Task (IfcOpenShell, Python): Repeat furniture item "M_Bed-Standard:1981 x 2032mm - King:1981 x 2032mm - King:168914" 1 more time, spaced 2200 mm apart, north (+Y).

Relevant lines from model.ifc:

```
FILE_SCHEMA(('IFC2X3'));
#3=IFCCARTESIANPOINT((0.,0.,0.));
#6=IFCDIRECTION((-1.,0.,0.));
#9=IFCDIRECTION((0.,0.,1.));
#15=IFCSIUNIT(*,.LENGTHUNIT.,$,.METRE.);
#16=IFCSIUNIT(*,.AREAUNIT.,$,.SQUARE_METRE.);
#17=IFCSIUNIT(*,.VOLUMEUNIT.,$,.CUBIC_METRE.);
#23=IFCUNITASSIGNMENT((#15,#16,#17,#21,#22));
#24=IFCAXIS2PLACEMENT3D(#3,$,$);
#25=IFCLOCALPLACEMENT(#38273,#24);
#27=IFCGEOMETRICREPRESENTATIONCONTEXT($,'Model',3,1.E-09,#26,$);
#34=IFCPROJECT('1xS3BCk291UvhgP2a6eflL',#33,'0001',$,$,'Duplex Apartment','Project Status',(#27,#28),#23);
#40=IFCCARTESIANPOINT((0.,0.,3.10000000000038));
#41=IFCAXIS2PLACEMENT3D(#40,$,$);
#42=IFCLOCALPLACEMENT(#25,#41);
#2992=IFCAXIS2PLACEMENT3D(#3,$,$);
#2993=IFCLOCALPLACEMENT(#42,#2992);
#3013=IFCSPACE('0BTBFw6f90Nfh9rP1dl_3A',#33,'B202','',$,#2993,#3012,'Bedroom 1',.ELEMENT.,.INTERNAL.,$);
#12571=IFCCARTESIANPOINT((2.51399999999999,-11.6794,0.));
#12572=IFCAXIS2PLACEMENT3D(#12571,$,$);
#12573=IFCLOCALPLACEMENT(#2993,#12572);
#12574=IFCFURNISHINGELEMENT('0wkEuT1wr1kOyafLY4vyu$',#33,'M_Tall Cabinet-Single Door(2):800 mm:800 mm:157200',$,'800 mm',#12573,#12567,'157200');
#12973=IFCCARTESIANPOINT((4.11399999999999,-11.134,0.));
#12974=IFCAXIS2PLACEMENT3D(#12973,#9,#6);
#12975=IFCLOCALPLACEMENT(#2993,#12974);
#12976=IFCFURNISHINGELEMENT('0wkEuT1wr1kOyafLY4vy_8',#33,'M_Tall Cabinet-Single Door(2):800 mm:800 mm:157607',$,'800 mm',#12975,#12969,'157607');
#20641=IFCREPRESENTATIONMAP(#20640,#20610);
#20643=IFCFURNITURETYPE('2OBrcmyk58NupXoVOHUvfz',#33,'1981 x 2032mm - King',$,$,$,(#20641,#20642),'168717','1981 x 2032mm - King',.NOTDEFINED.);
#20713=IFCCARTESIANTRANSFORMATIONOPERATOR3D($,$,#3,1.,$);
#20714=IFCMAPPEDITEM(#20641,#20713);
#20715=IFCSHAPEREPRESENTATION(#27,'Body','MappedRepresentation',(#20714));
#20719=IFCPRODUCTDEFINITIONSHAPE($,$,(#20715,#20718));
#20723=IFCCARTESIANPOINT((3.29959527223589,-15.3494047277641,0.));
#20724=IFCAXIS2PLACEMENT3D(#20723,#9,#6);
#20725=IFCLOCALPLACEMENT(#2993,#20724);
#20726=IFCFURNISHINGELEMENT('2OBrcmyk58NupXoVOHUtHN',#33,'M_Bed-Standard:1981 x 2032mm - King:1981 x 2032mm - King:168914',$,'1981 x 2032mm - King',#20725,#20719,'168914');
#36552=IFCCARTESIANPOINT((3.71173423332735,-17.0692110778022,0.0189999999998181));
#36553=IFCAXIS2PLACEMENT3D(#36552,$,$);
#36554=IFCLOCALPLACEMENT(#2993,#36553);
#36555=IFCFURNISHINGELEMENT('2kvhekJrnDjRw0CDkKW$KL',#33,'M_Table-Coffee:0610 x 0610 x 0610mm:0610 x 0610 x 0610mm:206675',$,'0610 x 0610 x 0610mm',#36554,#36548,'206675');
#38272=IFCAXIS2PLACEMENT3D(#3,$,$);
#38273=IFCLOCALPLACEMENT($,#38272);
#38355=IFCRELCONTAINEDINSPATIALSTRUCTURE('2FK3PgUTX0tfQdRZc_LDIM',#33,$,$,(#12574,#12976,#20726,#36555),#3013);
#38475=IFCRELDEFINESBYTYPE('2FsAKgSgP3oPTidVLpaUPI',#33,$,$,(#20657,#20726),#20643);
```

```python
import numpy as np
import ifcopenshell
import ifcopenshell.api.geometry
import ifcopenshell.api.root
import ifcopenshell.util.element
import ifcopenshell.util.placement

model = ifcopenshell.open("model.ifc")


def reuse_history(source, copy):
    """copy_class also copies each property set's owner history, people and application; keep the originals."""
    for rel in copy.IsDefinedBy:
        if rel.is_a("IfcRelDefinesByProperties") and (history := rel.RelatingPropertyDefinition.OwnerHistory):
            rel.RelatingPropertyDefinition.OwnerHistory = source.OwnerHistory
            ifcopenshell.util.element.remove_deep2(model, history)


source = model.by_guid("2OBrcmyk58NupXoVOHUtHN")
base = ifcopenshell.util.placement.get_local_placement(source.ObjectPlacement)
step = np.array([0.0, 1.0, 0.0]) * 2.2

for i in range(1, 2):
    copy = ifcopenshell.api.root.copy_class(model, product=source)
    copy.Representation = ifcopenshell.util.element.copy_deep(
        model, source.Representation, exclude=["IfcGeometricRepresentationContext", "IfcRepresentationMap"]
    )
    copy.Name = "M_Bed-Standard:1981 x 2032mm - King:1981 x 2032mm - King"
    copy.Tag = None
    reuse_history(source, copy)
    matrix = base.copy()
    matrix[:3, 3] += i * step
    print("added at", matrix[:3, 3].round(3) + 0.0)
    ifcopenshell.api.geometry.edit_object_placement(model, product=copy, matrix=matrix, is_si=False)

model.write("model_rev.ifc")
```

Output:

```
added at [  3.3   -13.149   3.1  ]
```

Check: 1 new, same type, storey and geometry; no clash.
